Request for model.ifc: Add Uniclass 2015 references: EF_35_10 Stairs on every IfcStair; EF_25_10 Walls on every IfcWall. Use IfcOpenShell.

First a look at what the model holds.

```python
import ifcopenshell

model = ifcopenshell.open("model.ifc")
print(model.schema)
print("classifications:", [c.Name for c in model.by_type("IfcClassification")])
for ifc_class in ("IfcDoor", "IfcRoof", "IfcStair", "IfcWall", "IfcWindow"):
    print(ifc_class, len(model.by_type(ifc_class)))
```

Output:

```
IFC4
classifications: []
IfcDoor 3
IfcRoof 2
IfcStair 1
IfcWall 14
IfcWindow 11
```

```python
import ifcopenshell
import ifcopenshell.api.classification

model = ifcopenshell.open("model.ifc")

system = ifcopenshell.api.classification.add_classification(model, classification="Uniclass 2015")

codes = {
    "IfcStair": ("EF_35_10", "Stairs"),
    "IfcWall": ("EF_25_10", "Walls"),
}
for ifc_class, (code, name) in codes.items():
    products = model.by_type(ifc_class)
    ifcopenshell.api.classification.add_reference(
        model, products=products, classification=system, identification=code, name=name
    )
    print(code, len(products))

model.write("model_rev.ifc")
```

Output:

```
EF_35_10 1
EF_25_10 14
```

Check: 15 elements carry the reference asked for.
